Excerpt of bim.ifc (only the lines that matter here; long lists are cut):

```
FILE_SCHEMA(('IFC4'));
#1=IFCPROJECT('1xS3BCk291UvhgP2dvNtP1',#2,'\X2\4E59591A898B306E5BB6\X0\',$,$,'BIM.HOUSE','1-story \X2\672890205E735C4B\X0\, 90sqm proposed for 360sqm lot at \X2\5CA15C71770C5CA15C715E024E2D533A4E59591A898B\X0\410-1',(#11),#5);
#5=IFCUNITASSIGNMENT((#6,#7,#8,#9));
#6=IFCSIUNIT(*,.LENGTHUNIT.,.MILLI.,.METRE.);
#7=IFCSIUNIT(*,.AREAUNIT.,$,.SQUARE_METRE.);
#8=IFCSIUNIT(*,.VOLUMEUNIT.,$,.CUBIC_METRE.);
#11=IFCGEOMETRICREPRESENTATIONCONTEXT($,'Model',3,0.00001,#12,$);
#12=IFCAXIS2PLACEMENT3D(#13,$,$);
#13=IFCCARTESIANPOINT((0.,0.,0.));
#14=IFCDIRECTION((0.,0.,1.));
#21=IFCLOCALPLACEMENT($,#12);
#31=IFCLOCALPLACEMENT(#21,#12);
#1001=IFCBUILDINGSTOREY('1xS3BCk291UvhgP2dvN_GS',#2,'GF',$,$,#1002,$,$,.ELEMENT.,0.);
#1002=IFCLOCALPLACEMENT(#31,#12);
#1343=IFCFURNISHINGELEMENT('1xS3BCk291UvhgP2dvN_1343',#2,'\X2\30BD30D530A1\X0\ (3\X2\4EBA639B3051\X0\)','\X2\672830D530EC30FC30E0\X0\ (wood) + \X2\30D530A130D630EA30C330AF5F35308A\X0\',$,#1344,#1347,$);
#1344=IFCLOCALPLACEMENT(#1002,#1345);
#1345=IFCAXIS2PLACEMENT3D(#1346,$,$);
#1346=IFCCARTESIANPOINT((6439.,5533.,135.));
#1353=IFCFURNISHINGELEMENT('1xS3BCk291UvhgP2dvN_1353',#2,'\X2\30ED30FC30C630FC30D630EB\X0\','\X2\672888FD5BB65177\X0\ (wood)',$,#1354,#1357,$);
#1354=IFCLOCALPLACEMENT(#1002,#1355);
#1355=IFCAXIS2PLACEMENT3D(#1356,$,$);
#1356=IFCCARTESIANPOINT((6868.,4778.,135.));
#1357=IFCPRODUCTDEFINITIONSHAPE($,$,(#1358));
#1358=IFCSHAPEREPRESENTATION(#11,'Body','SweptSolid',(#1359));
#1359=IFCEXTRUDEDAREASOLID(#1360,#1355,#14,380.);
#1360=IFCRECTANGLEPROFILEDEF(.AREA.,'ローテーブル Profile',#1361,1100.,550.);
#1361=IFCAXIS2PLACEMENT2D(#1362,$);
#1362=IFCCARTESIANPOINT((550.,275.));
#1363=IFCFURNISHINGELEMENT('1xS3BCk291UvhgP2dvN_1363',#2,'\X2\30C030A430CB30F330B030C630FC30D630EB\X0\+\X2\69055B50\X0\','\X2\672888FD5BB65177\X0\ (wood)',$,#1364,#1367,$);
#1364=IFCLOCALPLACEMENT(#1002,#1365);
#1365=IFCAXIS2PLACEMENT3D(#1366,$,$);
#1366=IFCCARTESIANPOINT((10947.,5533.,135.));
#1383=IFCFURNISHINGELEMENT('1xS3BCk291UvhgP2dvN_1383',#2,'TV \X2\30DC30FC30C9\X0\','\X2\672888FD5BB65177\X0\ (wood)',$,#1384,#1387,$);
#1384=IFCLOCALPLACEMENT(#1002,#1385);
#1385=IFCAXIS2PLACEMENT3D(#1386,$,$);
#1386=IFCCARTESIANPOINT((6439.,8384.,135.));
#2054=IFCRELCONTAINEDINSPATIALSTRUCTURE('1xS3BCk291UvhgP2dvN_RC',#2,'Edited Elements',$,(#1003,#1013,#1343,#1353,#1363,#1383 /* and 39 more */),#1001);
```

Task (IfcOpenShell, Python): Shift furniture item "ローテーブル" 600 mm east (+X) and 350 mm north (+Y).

```python
import ifcopenshell
import ifcopenshell.api.geometry
import ifcopenshell.util.placement
import ifcopenshell.util.unit

model = ifcopenshell.open("bim.ifc")
unit_scale = ifcopenshell.util.unit.calculate_unit_scale(model)

item = model.by_guid("1xS3BCk291UvhgP2dvN_1353")
matrix = ifcopenshell.util.placement.get_local_placement(item.ObjectPlacement)
matrix[0, 3] += 0.6 / unit_scale
matrix[1, 3] += 0.35 / unit_scale
ifcopenshell.api.geometry.edit_object_placement(model, product=item, matrix=matrix, is_si=False)

print(ifcopenshell.util.placement.get_local_placement(item.ObjectPlacement).round(3) + 0.0)

model.write("bim-out.ifc")
```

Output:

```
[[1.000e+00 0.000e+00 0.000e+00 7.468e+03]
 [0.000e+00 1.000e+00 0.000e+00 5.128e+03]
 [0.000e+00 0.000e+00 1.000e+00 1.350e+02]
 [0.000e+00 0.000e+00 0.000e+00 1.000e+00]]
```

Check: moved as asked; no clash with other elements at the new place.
